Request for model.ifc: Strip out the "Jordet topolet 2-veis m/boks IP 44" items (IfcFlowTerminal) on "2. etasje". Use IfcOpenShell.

First a look at what the model holds.

```python
import ifcopenshell
import ifcopenshell.util.element

model = ifcopenshell.open("model.ifc")
print(model.schema)
storey = next(s for s in model.by_type("IfcBuildingStorey") if s.Name == "2. etasje")
terminals = [e for e in ifcopenshell.util.element.get_decomposition(storey) if e.is_a("IfcFlowTerminal")]
seen = {}
for e in terminals:
    element_type = ifcopenshell.util.element.get_type(e)
    name = element_type.Name if element_type not in (None, e) else None
    seen[name] = seen.get(name, 0) + 1
for name, count in sorted(seen.items(), key=str):
    print(count, "x", name)
```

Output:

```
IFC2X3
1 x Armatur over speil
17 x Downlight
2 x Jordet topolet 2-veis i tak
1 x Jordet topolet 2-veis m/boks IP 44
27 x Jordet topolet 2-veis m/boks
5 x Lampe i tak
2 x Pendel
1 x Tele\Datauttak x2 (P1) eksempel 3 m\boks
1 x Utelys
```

```python
import ifcopenshell
import ifcopenshell.api.root
import ifcopenshell.util.element

model = ifcopenshell.open("model.ifc")

storey = next(s for s in model.by_type("IfcBuildingStorey") if s.Name == "2. etasje")
terminals = [e for e in ifcopenshell.util.element.get_decomposition(storey) if e.is_a("IfcFlowTerminal")]
targets = [e for e in terminals if (t := ifcopenshell.util.element.get_type(e)) not in (None, e) and t.Name == "Jordet topolet 2-veis m/boks IP 44"]

for e in targets:
    ifcopenshell.api.root.remove_product(model, product=e)
print(len(targets), "removed")

model.write("model_updated.ifc")
```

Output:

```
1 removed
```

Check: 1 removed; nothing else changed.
